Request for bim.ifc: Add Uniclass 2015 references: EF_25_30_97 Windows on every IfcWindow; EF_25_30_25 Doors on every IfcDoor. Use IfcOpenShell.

First a look at what the model holds.

```python
import ifcopenshell

model = ifcopenshell.open("bim.ifc")
print(model.schema)
print("classifications:", [c.Name for c in model.by_type("IfcClassification")])
for ifc_class in ("IfcDoor", "IfcRoof", "IfcStair", "IfcWall", "IfcWindow"):
    print(ifc_class, len(model.by_type(ifc_class)))
```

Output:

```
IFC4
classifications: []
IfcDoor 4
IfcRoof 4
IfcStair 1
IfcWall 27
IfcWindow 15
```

```python
import ifcopenshell
import ifcopenshell.api.classification

model = ifcopenshell.open("bim.ifc")

system = ifcopenshell.api.classification.add_classification(model, classification="Uniclass 2015")

codes = {
    "IfcWindow": ("EF_25_30_97", "Windows"),
    "IfcDoor": ("EF_25_30_25", "Doors"),
}
for ifc_class, (code, name) in codes.items():
    products = model.by_type(ifc_class)
    ifcopenshell.api.classification.add_reference(
        model, products=products, classification=system, identification=code, name=name
    )
    print(code, len(products))

model.write("bim_rev.ifc")
```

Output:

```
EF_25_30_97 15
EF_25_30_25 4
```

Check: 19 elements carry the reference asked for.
